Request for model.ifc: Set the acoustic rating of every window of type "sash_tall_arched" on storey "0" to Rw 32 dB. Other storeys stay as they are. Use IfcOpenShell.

First a look at what the model holds.

```python
import ifcopenshell
import ifcopenshell.util.element

model = ifcopenshell.open("model.ifc")
print(model.schema)
storey = next(s for s in model.by_type("IfcBuildingStorey") if s.Name == "0")
windows = [e for e in ifcopenshell.util.element.get_decomposition(storey) if e.is_a("IfcWindow")]
seen = {}
for e in windows:
    element_type = ifcopenshell.util.element.get_type(e)
    key = (element_type.Name if element_type != e and element_type else None, ifcopenshell.util.element.get_pset(e, "Pset_WindowCommon", "AcousticRating"))
    seen[key] = seen.get(key, 0) + 1
for (name, value), count in sorted(seen.items(), key=str):
    print(count, "x", name, "|", value)
```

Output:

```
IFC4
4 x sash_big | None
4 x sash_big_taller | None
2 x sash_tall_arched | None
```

```python
import ifcopenshell
import ifcopenshell.api.pset
import ifcopenshell.util.element

model = ifcopenshell.open("model.ifc")

storey = next(s for s in model.by_type("IfcBuildingStorey") if s.Name == "0")
windows = [e for e in ifcopenshell.util.element.get_decomposition(storey) if e.is_a("IfcWindow")]

count = 0
for e in windows:
    element_type = ifcopenshell.util.element.get_type(e)
    if element_type in (None, e) or element_type.Name != "sash_tall_arched":
        continue
    # add_pset returns the element's existing set when there is one.
    pset = ifcopenshell.api.pset.add_pset(model, product=e, name="Pset_WindowCommon")
    ifcopenshell.api.pset.edit_pset(model, pset=pset, properties={"AcousticRating": "Rw 32 dB"})
    count += 1

print(count, "windows updated")

model.write("model_edited.ifc")
```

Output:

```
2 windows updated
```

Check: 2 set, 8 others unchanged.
